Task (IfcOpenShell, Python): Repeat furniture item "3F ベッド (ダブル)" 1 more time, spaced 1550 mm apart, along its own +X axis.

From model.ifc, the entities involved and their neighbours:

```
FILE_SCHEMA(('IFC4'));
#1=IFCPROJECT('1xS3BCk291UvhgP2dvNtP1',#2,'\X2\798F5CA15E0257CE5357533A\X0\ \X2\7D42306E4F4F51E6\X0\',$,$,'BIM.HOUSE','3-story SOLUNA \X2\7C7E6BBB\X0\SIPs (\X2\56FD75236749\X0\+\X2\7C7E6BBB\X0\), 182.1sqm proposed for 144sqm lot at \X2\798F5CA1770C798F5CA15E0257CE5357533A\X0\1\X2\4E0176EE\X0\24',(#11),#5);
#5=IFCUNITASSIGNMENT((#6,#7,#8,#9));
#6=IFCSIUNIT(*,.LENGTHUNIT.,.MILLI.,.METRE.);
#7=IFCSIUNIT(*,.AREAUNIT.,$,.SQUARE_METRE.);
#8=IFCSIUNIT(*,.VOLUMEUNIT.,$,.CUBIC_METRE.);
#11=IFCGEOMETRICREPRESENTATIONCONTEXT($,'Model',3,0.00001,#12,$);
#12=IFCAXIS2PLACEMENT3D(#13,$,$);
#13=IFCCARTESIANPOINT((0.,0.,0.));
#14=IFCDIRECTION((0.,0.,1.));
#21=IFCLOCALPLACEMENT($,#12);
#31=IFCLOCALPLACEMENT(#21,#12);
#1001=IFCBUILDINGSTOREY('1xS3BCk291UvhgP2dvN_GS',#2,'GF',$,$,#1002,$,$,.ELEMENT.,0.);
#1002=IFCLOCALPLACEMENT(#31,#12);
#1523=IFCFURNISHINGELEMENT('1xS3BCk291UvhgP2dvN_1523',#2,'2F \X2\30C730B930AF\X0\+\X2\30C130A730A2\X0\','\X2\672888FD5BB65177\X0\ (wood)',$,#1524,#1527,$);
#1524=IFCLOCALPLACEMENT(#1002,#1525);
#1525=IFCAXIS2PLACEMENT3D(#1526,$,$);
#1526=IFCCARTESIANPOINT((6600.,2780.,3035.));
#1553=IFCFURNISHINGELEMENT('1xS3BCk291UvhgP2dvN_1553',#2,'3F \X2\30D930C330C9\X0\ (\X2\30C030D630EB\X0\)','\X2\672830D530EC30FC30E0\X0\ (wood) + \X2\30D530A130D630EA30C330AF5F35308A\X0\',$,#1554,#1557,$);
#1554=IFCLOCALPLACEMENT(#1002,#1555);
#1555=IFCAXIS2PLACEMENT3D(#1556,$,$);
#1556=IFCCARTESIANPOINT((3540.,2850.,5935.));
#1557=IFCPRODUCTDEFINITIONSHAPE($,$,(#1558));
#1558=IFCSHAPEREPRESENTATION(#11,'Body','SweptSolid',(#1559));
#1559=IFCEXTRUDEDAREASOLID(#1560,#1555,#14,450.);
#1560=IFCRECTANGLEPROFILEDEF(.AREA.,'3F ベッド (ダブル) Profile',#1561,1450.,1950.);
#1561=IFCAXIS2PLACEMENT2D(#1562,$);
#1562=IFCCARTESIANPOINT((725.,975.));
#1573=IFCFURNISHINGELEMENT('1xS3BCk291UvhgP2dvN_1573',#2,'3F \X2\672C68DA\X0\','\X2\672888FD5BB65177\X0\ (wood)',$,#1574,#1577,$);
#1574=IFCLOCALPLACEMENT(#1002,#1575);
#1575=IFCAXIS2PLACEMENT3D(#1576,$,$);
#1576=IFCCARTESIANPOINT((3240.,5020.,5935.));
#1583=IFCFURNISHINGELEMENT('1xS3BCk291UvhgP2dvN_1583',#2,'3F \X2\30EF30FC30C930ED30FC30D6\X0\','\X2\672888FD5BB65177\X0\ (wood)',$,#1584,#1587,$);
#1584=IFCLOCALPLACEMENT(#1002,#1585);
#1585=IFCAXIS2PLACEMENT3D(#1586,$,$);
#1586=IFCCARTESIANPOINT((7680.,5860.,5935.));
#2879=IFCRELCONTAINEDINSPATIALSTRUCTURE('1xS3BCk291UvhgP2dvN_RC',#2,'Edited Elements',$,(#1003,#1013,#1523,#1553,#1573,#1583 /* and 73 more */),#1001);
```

```python
import ifcopenshell
import ifcopenshell.api.geometry
import ifcopenshell.api.root
import ifcopenshell.util.element
import ifcopenshell.util.placement
import ifcopenshell.util.unit

model = ifcopenshell.open("model.ifc")
unit_scale = ifcopenshell.util.unit.calculate_unit_scale(model)


def reuse_history(source, copy):
    """copy_class also copies each property set's owner history, people and application; keep the originals."""
    for rel in copy.IsDefinedBy:
        if rel.is_a("IfcRelDefinesByProperties") and (history := rel.RelatingPropertyDefinition.OwnerHistory):
            rel.RelatingPropertyDefinition.OwnerHistory = source.OwnerHistory
            ifcopenshell.util.element.remove_deep2(model, history)


source = model.by_guid("1xS3BCk291UvhgP2dvN_1553")
base = ifcopenshell.util.placement.get_local_placement(source.ObjectPlacement)
step = base[:3, 0] * 1.55 / unit_scale

for i in range(1, 2):
    copy = ifcopenshell.api.root.copy_class(model, product=source)
    copy.Representation = ifcopenshell.util.element.copy_deep(
        model, source.Representation, exclude=["IfcGeometricRepresentationContext", "IfcRepresentationMap"]
    )
    reuse_history(source, copy)
    matrix = base.copy()
    matrix[:3, 3] += i * step
    print("added at", matrix[:3, 3].round(3) + 0.0)
    ifcopenshell.api.geometry.edit_object_placement(model, product=copy, matrix=matrix, is_si=False)

model.write("model_rev.ifc")
```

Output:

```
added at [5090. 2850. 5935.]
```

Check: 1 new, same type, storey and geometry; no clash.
